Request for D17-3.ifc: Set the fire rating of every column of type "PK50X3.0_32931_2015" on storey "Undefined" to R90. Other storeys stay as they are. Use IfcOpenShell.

First a look at what the model holds.

```python
import ifcopenshell
import ifcopenshell.util.element

model = ifcopenshell.open("D17-3.ifc")
print(model.schema)
storey = next(s for s in model.by_type("IfcBuildingStorey") if s.Name == "Undefined")
columns = [e for e in ifcopenshell.util.element.get_decomposition(storey) if e.is_a("IfcColumn")]
seen = {}
for e in columns:
    element_type = ifcopenshell.util.element.get_type(e)
    key = (element_type.Name if element_type != e and element_type else None, ifcopenshell.util.element.get_pset(e, "Pset_ColumnCommon", "FireRating"))
    seen[key] = seen.get(key, 0) + 1
for (name, value), count in sorted(seen.items(), key=str):
    print(count, "x", name, "|", value)
```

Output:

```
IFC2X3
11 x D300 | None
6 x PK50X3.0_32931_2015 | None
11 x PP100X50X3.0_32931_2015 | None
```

```python
import ifcopenshell
import ifcopenshell.api.pset
import ifcopenshell.util.element

model = ifcopenshell.open("D17-3.ifc")

storey = next(s for s in model.by_type("IfcBuildingStorey") if s.Name == "Undefined")
columns = [e for e in ifcopenshell.util.element.get_decomposition(storey) if e.is_a("IfcColumn")]

count = 0
for e in columns:
    element_type = ifcopenshell.util.element.get_type(e)
    if element_type in (None, e) or element_type.Name != "PK50X3.0_32931_2015":
        continue
    found = ifcopenshell.util.element.get_pset(e, "Pset_ColumnCommon", should_inherit=False)
    if found:
        pset = model.by_id(found["id"])
        if len(ifcopenshell.util.element.get_elements_by_pset(pset)) > 1:
            pset = ifcopenshell.api.pset.unshare_pset(model, products=[e], pset=pset)[0]
    else:
        pset = ifcopenshell.api.pset.add_pset(model, product=e, name="Pset_ColumnCommon")
    ifcopenshell.api.pset.edit_pset(model, pset=pset, properties={"FireRating": "R90"})
    count += 1

print(count, "columns updated")

model.write("D17-3_edited.ifc")
```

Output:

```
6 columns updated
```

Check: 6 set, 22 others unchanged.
